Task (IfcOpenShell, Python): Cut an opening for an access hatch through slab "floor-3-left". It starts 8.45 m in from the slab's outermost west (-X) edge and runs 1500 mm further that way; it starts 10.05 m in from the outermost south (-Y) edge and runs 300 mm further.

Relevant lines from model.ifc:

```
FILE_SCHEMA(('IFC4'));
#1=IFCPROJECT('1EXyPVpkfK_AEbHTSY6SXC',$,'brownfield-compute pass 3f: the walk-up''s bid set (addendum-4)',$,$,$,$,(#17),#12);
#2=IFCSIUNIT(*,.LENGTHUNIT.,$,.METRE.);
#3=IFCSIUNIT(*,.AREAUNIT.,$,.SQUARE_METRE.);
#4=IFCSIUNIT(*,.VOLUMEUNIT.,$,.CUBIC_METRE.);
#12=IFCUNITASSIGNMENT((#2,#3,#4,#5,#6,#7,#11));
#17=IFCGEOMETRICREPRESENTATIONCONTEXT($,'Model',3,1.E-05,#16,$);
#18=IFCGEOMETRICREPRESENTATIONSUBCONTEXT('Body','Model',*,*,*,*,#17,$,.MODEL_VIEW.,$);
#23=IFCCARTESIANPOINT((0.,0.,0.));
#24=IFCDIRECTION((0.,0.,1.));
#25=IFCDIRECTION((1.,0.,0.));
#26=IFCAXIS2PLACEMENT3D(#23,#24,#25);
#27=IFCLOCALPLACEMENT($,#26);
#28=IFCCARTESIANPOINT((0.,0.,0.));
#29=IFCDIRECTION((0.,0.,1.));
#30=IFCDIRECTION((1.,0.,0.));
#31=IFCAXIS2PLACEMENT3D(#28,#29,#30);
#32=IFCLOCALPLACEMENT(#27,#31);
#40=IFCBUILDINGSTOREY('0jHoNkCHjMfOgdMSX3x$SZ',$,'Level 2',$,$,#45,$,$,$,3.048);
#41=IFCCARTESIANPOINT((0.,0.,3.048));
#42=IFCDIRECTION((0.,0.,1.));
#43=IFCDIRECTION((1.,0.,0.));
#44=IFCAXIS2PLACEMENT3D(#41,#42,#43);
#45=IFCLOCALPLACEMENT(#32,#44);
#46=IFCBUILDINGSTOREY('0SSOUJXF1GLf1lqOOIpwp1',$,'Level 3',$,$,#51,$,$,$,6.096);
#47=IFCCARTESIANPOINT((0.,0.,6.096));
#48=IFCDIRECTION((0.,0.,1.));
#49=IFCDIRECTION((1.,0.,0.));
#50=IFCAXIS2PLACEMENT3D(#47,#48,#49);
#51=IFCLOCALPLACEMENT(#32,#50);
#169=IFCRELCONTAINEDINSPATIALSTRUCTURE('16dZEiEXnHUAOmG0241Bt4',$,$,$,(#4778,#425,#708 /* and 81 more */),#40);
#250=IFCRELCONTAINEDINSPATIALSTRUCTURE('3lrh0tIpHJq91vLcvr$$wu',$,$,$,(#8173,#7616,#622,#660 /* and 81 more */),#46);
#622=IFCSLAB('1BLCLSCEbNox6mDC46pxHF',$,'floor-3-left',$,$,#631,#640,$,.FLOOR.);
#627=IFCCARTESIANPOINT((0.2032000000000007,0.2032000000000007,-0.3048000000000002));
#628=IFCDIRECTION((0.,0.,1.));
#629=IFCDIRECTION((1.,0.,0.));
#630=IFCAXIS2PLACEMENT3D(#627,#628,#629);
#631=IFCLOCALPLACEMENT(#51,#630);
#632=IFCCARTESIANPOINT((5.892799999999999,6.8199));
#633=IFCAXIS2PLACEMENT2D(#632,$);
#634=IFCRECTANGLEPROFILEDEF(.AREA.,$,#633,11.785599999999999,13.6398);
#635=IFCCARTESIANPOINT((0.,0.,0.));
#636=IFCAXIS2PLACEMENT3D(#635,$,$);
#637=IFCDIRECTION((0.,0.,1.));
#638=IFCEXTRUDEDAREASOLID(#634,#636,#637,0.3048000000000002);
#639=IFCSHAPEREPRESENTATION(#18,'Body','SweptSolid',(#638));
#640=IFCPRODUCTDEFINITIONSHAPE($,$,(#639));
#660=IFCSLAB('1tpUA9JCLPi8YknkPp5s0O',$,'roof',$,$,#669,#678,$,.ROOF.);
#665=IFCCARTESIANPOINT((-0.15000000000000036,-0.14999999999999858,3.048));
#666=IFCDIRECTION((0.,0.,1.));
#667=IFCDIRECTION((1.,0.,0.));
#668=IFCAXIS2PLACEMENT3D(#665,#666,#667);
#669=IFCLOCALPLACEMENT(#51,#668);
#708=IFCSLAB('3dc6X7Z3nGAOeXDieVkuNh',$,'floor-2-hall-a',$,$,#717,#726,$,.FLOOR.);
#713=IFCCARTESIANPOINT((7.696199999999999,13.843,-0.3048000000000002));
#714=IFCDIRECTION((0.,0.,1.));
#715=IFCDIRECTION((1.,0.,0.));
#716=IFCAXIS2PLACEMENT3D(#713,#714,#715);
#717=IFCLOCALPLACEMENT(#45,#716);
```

```python
import numpy as np
import ifcopenshell
import ifcopenshell.api.feature
import ifcopenshell.api.geometry
import ifcopenshell.api.root
import ifcopenshell.geom
import ifcopenshell.util.placement
import ifcopenshell.util.representation
import ifcopenshell.util.shape
import ifcopenshell.util.unit

model = ifcopenshell.open("model.ifc")
unit_scale = ifcopenshell.util.unit.calculate_unit_scale(model)
settings = ifcopenshell.geom.settings()


def volume(element):
    """Net volume in cubic metres, openings subtracted."""
    shape = ifcopenshell.geom.create_shape(settings, element)
    return ifcopenshell.util.shape.get_volume(shape.geometry)


slab = model.by_guid("1BLCLSCEbNox6mDC46pxHF")
before = volume(slab)

# Extent in the slab's own axes, in metres. The edges named are its -X and -Y sides.
slab_shape = ifcopenshell.geom.create_shape(settings, slab)
vertices = ifcopenshell.util.shape.get_vertices(slab_shape.geometry)
x_min, y_min, bottom = vertices.min(axis=0)
top = vertices[:, 2].max()

opening = ifcopenshell.api.root.create_entity(model, ifc_class="IfcOpeningElement", name="Access hatch opening", predefined_type="OPENING")
context = ifcopenshell.util.representation.get_context(model, "Model", "Body", "MODEL_VIEW")
width, depth = 1.5, 0.3
outline = [(0.0, 0.0), (width, 0.0), (width, depth), (0.0, depth), (0.0, 0.0)]
# Overshoot both faces by 50 mm so the cut is clean.
shape = ifcopenshell.api.geometry.add_slab_representation(
    model, context=context, depth=top - bottom + 0.1, polyline=outline
)
ifcopenshell.api.geometry.assign_representation(model, product=opening, representation=shape)

matrix = ifcopenshell.util.placement.get_local_placement(slab.ObjectPlacement)
matrix[:, 3] = matrix @ np.append(np.array([x_min + 8.45, y_min + 10.05, bottom - 0.05]) / unit_scale, 1.0)
ifcopenshell.api.geometry.edit_object_placement(model, product=opening, matrix=matrix, is_si=False)
ifcopenshell.api.feature.add_feature(model, feature=opening, element=slab)

after = volume(slab)

print(f"slab volume {before:.3f} -> {after:.3f} m3")

model.write("model_updated.ifc")
```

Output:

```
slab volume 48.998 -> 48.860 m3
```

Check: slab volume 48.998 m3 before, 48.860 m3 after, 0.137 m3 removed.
